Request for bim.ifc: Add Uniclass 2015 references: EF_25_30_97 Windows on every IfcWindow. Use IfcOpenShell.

First a look at what the model holds.

```python
import ifcopenshell

model = ifcopenshell.open("bim.ifc")
print(model.schema)
print("classifications:", [c.Name for c in model.by_type("IfcClassification")])
for ifc_class in ("IfcDoor", "IfcRoof", "IfcStair", "IfcWall", "IfcWindow"):
    print(ifc_class, len(model.by_type(ifc_class)))
```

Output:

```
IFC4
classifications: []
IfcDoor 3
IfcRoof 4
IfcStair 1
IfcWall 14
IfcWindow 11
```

```python
import ifcopenshell
import ifcopenshell.api.classification

model = ifcopenshell.open("bim.ifc")

system = ifcopenshell.api.classification.add_classification(model, classification="Uniclass 2015")

codes = {
    "IfcWindow": ("EF_25_30_97", "Windows"),
}
for ifc_class, (code, name) in codes.items():
    products = model.by_type(ifc_class)
    ifcopenshell.api.classification.add_reference(
        model, products=products, classification=system, identification=code, name=name
    )
    print(code, len(products))

model.write("bim_rev.ifc")
```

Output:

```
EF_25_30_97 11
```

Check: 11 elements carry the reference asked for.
